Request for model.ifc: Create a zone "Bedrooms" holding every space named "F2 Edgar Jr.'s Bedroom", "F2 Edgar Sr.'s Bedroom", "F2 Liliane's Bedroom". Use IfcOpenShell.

First a look at what the model holds.

```python
import ifcopenshell

model = ifcopenshell.open("model.ifc")
print(model.schema)
seen = {}
for space in model.by_type("IfcSpace"):
    seen[space.Name] = seen.get(space.Name, 0) + 1
for name, count in sorted(seen.items(), key=str):
    print(count, "x", name)
print("zones:", [z.Name for z in model.by_type("IfcZone")][:20])
```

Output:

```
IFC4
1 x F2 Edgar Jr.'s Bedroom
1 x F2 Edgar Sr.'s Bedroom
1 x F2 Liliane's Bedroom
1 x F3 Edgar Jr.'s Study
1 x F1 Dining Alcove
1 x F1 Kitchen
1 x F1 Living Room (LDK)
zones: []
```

```python
import ifcopenshell
import ifcopenshell.api.group
import ifcopenshell.api.root

model = ifcopenshell.open("model.ifc")

names = {"F2 Edgar Jr.'s Bedroom", "F2 Edgar Sr.'s Bedroom", "F2 Liliane's Bedroom"}
spaces = [s for s in model.by_type("IfcSpace") if s.Name in names]

zone = ifcopenshell.api.root.create_entity(model, ifc_class="IfcZone", name="Bedrooms")
ifcopenshell.api.group.assign_group(model, products=spaces, group=zone)
print(len(spaces), "spaces in", zone.Name)

model.write("model_v2.ifc")
```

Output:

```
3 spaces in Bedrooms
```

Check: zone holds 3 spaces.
